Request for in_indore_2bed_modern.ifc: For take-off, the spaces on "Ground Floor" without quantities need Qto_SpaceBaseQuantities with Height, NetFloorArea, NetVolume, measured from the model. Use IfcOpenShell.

First a look at what the model holds.

```python
import ifcopenshell
import ifcopenshell.util.element
import ifcopenshell.util.unit

model = ifcopenshell.open("in_indore_2bed_modern.ifc")
print(model.schema)
for unit_type in ("LENGTHUNIT", "AREAUNIT", "VOLUMEUNIT"):
    print(unit_type, ifcopenshell.util.unit.calculate_unit_scale(model, unit_type))
storey = next(s for s in model.by_type("IfcBuildingStorey") if s.Name == "Ground Floor")
spaces = [e for e in ifcopenshell.util.element.get_decomposition(storey) if e.is_a("IfcSpace")]
for e in sorted(spaces, key=lambda e: e.id()):
    print(e.id(), e.is_a(), e.Name, list(ifcopenshell.util.element.get_psets(e, qtos_only=True)), sep=" | ")
```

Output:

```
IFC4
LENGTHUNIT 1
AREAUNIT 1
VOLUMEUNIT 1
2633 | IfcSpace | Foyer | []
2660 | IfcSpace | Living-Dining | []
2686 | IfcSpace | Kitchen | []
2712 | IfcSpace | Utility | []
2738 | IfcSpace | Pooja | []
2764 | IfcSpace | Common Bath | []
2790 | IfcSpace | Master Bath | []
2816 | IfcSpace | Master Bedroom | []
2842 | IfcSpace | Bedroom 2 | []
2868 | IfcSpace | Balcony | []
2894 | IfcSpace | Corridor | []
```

```python
import ifcopenshell
import ifcopenshell.api.pset
import ifcopenshell.geom
import ifcopenshell.util.element
import ifcopenshell.util.shape
import ifcopenshell.util.unit

model = ifcopenshell.open("in_indore_2bed_modern.ifc")
unit_scale = ifcopenshell.util.unit.calculate_unit_scale(model)
area_scale = ifcopenshell.util.unit.calculate_unit_scale(model, "AREAUNIT")
volume_scale = ifcopenshell.util.unit.calculate_unit_scale(model, "VOLUMEUNIT")
settings = ifcopenshell.geom.settings()

storey = next(s for s in model.by_type("IfcBuildingStorey") if s.Name == "Ground Floor")
spaces = [e for e in ifcopenshell.util.element.get_decomposition(storey) if e.is_a("IfcSpace")]

for e in sorted(spaces, key=lambda e: e.id()):
    if ifcopenshell.util.element.get_psets(e, qtos_only=True, should_inherit=False):
        continue
    # Geometry comes back in metres, in the element's own axes.
    shape = ifcopenshell.geom.create_shape(settings, e)
    values = {
        "Height": ifcopenshell.util.shape.get_z(shape.geometry) / unit_scale,
        "NetFloorArea": ifcopenshell.util.shape.get_footprint_area(shape.geometry) / area_scale,
        "NetVolume": ifcopenshell.util.shape.get_volume(shape.geometry) / volume_scale,
    }
    qto = ifcopenshell.api.pset.add_qto(model, product=e, name="Qto_SpaceBaseQuantities")
    ifcopenshell.api.pset.edit_qto(model, qto=qto, properties=values)
    print(e.id(), {k: round(v, 3) for k, v in values.items()})

model.write("in_indore_2bed_modern_v2.ifc")
```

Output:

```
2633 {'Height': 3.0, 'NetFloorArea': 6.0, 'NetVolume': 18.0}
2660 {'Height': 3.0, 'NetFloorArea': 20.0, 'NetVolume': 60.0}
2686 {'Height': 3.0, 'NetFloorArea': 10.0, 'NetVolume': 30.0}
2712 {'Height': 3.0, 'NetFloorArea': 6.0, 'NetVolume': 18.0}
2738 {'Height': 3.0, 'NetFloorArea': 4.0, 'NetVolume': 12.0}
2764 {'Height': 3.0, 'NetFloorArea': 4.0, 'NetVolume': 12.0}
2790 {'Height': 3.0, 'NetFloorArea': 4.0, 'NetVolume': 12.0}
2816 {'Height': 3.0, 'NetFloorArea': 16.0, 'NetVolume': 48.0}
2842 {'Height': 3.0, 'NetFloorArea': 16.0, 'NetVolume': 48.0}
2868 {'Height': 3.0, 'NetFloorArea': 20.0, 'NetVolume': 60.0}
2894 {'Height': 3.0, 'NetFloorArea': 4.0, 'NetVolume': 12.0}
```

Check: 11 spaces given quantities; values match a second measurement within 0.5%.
